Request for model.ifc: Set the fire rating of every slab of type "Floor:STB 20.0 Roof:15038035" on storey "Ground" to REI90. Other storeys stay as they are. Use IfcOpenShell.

First a look at what the model holds.

```python
import ifcopenshell
import ifcopenshell.util.element

model = ifcopenshell.open("model.ifc")
print(model.schema)
storey = next(s for s in model.by_type("IfcBuildingStorey") if s.Name == "Ground")
slabs = [e for e in ifcopenshell.util.element.get_decomposition(storey) if e.is_a("IfcSlab")]
seen = {}
for e in slabs:
    element_type = ifcopenshell.util.element.get_type(e)
    key = (element_type.Name if element_type != e and element_type else None, ifcopenshell.util.element.get_pset(e, "Pset_SlabCommon", "FireRating"))
    seen[key] = seen.get(key, 0) + 1
for (name, value), count in sorted(seen.items(), key=str):
    print(count, "x", name, "|", value)
```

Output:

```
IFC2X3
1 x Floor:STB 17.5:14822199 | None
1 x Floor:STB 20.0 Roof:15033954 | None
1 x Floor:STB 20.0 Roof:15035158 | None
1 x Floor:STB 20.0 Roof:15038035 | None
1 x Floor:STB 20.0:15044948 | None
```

```python
import ifcopenshell
import ifcopenshell.api.pset
import ifcopenshell.util.element

model = ifcopenshell.open("model.ifc")

storey = next(s for s in model.by_type("IfcBuildingStorey") if s.Name == "Ground")
slabs = [e for e in ifcopenshell.util.element.get_decomposition(storey) if e.is_a("IfcSlab")]

count = 0
for e in slabs:
    element_type = ifcopenshell.util.element.get_type(e)
    if element_type in (None, e) or element_type.Name != "Floor:STB 20.0 Roof:15038035":
        continue
    # add_pset returns the element's existing set when there is one.
    pset = ifcopenshell.api.pset.add_pset(model, product=e, name="Pset_SlabCommon")
    ifcopenshell.api.pset.edit_pset(model, pset=pset, properties={"FireRating": "REI90"})
    count += 1

print(count, "slabs updated")

model.write("model_v2.ifc")
```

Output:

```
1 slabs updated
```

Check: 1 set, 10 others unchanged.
